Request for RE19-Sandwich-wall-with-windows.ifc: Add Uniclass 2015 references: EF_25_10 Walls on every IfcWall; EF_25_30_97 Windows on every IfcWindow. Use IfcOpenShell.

First a look at what the model holds.

```python
import ifcopenshell

model = ifcopenshell.open("RE19-Sandwich-wall-with-windows.ifc")
print(model.schema)
print("classifications:", [c.Name for c in model.by_type("IfcClassification")])
for ifc_class in ("IfcDoor", "IfcRoof", "IfcStair", "IfcWall", "IfcWindow"):
    print(ifc_class, len(model.by_type(ifc_class)))
```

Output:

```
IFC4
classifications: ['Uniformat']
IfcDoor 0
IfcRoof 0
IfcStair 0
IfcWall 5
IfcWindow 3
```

```python
import ifcopenshell
import ifcopenshell.api.classification

model = ifcopenshell.open("RE19-Sandwich-wall-with-windows.ifc")

system = ifcopenshell.api.classification.add_classification(model, classification="Uniclass 2015")

codes = {
    "IfcWall": ("EF_25_10", "Walls"),
    "IfcWindow": ("EF_25_30_97", "Windows"),
}
for ifc_class, (code, name) in codes.items():
    products = model.by_type(ifc_class)
    ifcopenshell.api.classification.add_reference(
        model, products=products, classification=system, identification=code, name=name
    )
    print(code, len(products))

model.write("RE19-Sandwich-wall-with-windows_updated.ifc")
```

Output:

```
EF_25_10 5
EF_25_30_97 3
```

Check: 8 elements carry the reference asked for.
